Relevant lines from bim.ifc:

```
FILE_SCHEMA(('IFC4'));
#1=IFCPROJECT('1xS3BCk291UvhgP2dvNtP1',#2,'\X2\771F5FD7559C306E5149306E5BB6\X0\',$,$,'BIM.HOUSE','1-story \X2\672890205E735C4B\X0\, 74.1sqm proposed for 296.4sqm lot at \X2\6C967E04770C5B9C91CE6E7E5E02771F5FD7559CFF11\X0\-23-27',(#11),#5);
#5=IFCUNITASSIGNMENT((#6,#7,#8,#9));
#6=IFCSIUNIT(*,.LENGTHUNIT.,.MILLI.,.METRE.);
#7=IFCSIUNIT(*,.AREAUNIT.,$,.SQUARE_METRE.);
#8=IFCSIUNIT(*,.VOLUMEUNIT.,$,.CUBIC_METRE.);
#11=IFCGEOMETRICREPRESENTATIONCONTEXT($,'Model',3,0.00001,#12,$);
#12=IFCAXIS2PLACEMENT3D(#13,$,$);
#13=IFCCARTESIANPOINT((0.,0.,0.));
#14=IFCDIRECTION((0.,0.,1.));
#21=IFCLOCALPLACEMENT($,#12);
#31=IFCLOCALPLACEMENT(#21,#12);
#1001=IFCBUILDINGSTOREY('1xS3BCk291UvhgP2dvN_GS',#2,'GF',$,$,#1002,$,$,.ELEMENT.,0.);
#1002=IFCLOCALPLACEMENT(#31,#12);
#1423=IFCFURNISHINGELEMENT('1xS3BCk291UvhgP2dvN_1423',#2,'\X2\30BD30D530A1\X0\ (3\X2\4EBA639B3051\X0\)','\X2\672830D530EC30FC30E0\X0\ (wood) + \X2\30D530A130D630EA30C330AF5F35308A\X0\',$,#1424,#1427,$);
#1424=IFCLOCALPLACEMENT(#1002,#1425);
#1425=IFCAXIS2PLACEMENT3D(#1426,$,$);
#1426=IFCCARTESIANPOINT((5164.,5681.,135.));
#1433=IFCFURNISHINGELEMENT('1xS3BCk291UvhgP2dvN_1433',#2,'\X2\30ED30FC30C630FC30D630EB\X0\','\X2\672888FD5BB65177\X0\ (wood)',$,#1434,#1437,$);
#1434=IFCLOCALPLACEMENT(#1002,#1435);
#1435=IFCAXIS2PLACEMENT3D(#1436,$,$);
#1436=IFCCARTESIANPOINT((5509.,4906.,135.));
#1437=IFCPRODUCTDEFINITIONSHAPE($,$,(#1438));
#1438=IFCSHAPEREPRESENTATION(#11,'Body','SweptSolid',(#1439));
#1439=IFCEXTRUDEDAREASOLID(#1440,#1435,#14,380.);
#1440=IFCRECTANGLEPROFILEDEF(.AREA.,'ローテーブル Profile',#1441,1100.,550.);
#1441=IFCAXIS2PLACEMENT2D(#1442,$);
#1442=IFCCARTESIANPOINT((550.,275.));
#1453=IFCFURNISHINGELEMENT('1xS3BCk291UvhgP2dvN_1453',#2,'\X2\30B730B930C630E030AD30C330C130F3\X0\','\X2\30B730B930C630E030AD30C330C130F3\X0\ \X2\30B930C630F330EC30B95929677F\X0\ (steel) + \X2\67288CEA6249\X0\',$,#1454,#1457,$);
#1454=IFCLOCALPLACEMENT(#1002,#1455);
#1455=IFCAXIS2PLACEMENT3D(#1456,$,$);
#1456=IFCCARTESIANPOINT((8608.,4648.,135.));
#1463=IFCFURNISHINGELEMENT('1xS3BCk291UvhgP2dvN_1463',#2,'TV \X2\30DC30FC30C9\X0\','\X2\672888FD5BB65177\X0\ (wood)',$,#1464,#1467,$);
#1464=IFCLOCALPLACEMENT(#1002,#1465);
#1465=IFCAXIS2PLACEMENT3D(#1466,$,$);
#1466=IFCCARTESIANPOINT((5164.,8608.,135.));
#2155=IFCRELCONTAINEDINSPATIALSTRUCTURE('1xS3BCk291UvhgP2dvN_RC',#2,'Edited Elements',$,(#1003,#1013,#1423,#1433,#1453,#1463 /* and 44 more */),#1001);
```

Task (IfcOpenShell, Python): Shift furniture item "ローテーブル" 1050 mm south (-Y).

```python
import ifcopenshell
import ifcopenshell.api.geometry
import ifcopenshell.util.placement
import ifcopenshell.util.unit

model = ifcopenshell.open("bim.ifc")
unit_scale = ifcopenshell.util.unit.calculate_unit_scale(model)

item = model.by_guid("1xS3BCk291UvhgP2dvN_1433")
matrix = ifcopenshell.util.placement.get_local_placement(item.ObjectPlacement)
matrix[1, 3] -= 1.05 / unit_scale
ifcopenshell.api.geometry.edit_object_placement(model, product=item, matrix=matrix, is_si=False)

print(ifcopenshell.util.placement.get_local_placement(item.ObjectPlacement).round(3) + 0.0)

model.write("bim-out.ifc")
```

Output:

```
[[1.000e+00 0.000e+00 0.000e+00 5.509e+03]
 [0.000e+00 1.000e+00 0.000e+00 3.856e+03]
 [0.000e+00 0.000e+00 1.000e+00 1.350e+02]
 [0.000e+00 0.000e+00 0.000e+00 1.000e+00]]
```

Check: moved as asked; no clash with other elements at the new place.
